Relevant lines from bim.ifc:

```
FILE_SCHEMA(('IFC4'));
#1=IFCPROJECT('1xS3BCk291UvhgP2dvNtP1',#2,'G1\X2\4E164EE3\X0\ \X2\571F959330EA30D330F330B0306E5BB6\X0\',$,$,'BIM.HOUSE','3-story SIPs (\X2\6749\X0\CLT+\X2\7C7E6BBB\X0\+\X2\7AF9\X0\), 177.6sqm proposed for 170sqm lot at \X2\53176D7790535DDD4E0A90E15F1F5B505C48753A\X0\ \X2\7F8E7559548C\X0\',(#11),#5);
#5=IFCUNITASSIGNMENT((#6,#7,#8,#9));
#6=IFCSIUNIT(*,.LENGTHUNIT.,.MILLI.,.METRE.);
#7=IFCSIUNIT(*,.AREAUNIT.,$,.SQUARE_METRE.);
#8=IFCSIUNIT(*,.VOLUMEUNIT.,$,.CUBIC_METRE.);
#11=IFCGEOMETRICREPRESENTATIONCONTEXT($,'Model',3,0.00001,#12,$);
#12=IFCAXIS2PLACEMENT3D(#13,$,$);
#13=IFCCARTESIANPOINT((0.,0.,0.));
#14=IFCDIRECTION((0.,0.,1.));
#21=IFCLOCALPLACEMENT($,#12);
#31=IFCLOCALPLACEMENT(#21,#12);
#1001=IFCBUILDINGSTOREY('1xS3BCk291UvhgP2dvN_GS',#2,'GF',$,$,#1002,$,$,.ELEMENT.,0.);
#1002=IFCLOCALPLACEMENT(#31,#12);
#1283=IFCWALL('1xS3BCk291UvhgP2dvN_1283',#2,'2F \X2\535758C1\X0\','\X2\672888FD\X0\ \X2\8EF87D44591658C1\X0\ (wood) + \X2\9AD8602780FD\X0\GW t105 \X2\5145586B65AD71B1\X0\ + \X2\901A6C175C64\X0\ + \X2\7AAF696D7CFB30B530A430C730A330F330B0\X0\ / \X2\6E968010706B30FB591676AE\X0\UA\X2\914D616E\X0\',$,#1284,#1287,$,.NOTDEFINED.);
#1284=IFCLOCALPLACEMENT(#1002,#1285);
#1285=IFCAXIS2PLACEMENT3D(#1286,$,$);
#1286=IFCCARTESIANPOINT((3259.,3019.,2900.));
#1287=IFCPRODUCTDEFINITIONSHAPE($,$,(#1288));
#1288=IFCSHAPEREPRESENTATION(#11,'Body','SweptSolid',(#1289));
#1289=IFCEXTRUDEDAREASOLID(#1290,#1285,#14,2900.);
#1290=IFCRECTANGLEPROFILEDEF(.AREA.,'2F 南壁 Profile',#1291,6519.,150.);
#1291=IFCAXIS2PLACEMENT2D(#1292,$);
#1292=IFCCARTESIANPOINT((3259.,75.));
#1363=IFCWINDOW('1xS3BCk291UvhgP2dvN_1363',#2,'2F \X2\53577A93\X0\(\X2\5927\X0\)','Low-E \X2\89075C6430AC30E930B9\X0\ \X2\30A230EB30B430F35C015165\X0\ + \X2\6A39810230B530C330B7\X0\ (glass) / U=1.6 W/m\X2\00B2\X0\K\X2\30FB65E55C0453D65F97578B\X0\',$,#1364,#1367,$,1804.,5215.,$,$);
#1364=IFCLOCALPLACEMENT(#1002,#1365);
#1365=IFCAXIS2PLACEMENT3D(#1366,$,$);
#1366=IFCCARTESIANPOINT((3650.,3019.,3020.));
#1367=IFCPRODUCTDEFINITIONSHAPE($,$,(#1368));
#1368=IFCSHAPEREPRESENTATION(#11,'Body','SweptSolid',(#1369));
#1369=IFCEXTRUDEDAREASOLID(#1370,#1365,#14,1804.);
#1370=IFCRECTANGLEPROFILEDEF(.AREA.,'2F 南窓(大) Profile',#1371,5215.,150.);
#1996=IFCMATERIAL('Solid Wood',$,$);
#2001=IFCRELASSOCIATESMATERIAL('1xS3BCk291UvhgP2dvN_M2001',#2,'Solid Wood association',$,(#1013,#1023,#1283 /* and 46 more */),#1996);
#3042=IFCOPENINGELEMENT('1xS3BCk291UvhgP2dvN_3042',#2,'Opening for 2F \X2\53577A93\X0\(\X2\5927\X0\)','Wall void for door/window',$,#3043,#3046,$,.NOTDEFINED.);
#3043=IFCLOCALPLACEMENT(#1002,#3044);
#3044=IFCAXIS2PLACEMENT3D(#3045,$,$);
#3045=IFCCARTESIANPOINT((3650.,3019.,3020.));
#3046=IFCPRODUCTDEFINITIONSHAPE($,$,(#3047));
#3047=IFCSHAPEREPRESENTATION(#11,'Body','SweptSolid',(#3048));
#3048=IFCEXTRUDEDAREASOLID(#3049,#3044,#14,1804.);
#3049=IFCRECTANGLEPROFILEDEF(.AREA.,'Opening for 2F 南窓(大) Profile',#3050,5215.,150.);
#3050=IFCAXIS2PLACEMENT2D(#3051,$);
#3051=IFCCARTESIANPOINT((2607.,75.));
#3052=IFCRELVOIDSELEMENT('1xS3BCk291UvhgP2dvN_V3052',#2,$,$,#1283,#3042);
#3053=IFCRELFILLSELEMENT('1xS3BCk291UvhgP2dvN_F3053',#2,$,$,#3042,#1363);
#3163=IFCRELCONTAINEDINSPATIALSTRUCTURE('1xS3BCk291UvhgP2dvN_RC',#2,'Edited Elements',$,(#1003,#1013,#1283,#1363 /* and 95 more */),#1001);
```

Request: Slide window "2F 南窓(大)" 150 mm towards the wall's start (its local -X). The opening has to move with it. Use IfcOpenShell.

```python
import ifcopenshell
import ifcopenshell.api.geometry
import ifcopenshell.util.placement
import ifcopenshell.util.unit

model = ifcopenshell.open("bim.ifc")
unit_scale = ifcopenshell.util.unit.calculate_unit_scale(model)

window = model.by_id(1363)
opening = window.FillsVoids[0].RelatingOpeningElement
wall = opening.VoidsElements[0].RelatingBuildingElement

wall_matrix = ifcopenshell.util.placement.get_local_placement(wall.ObjectPlacement)
shift = wall_matrix[:3, 0] * -0.15 / unit_scale
before = ifcopenshell.util.placement.get_local_placement(window.ObjectPlacement)[:3, 3].copy()

# The window is not placed relative to its opening, so move both.
for product in (opening, window):
    matrix = ifcopenshell.util.placement.get_local_placement(product.ObjectPlacement)
    matrix[:3, 3] += shift
    ifcopenshell.api.geometry.edit_object_placement(model, product=product, matrix=matrix, is_si=False)

after = ifcopenshell.util.placement.get_local_placement(window.ObjectPlacement)[:3, 3]
print("window moved by", (after - before).round(3) + 0.0)

model.write("bim_updated.ifc")
```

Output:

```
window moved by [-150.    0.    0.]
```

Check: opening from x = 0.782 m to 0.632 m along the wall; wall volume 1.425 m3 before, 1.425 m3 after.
